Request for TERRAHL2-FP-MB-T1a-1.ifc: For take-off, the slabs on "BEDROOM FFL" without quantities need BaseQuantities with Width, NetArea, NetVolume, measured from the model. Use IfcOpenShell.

First a look at what the model holds.

```python
import ifcopenshell
import ifcopenshell.util.element
import ifcopenshell.util.unit

model = ifcopenshell.open("TERRAHL2-FP-MB-T1a-1.ifc")
print(model.schema)
for unit_type in ("LENGTHUNIT", "AREAUNIT", "VOLUMEUNIT"):
    print(unit_type, ifcopenshell.util.unit.calculate_unit_scale(model, unit_type))
storey = next(s for s in model.by_type("IfcBuildingStorey") if s.Name == "BEDROOM FFL")
slabs = [e for e in ifcopenshell.util.element.get_decomposition(storey) if e.is_a("IfcSlab")]
for e in sorted(slabs, key=lambda e: e.id()):
    print(e.id(), e.is_a(), e.Name, list(ifcopenshell.util.element.get_psets(e, qtos_only=True)), sep=" | ")
```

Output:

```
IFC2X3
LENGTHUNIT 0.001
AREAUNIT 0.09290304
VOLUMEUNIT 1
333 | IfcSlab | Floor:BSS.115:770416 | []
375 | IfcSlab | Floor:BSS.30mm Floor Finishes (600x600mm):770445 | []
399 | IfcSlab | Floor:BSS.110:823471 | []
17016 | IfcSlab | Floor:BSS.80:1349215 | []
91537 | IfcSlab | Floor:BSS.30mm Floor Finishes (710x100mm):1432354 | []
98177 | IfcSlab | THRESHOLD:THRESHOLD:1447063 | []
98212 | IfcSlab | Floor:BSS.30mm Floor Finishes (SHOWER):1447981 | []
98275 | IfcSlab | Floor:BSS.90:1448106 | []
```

```python
import ifcopenshell
import ifcopenshell.api.pset
import ifcopenshell.geom
import ifcopenshell.util.element
import ifcopenshell.util.shape
import ifcopenshell.util.unit

model = ifcopenshell.open("TERRAHL2-FP-MB-T1a-1.ifc")
unit_scale = ifcopenshell.util.unit.calculate_unit_scale(model)
area_scale = ifcopenshell.util.unit.calculate_unit_scale(model, "AREAUNIT")
volume_scale = ifcopenshell.util.unit.calculate_unit_scale(model, "VOLUMEUNIT")
settings = ifcopenshell.geom.settings()

storey = next(s for s in model.by_type("IfcBuildingStorey") if s.Name == "BEDROOM FFL")
slabs = [e for e in ifcopenshell.util.element.get_decomposition(storey) if e.is_a("IfcSlab")]

for e in sorted(slabs, key=lambda e: e.id()):
    if ifcopenshell.util.element.get_psets(e, qtos_only=True, should_inherit=False):
        continue
    # Geometry comes back in metres, in the element's own axes.
    shape = ifcopenshell.geom.create_shape(settings, e)
    values = {
        "Width": ifcopenshell.util.shape.get_z(shape.geometry) / unit_scale,
        "NetArea": ifcopenshell.util.shape.get_footprint_area(shape.geometry) / area_scale,
        "NetVolume": ifcopenshell.util.shape.get_volume(shape.geometry) / volume_scale,
    }
    qto = ifcopenshell.api.pset.add_qto(model, product=e, name="BaseQuantities")
    ifcopenshell.api.pset.edit_qto(model, qto=qto, properties=values)
    print(e.id(), {k: round(v, 3) for k, v in values.items()})

model.write("TERRAHL2-FP-MB-T1a-1_updated.ifc")
```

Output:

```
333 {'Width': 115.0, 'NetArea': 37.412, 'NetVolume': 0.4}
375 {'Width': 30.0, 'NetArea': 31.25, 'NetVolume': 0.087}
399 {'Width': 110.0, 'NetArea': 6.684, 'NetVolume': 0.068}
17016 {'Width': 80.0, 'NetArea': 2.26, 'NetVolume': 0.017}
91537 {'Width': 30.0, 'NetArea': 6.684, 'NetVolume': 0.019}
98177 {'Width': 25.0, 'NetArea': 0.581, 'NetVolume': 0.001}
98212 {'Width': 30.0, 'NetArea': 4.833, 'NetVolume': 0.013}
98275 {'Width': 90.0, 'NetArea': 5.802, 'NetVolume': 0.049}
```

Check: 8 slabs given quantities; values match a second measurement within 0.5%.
